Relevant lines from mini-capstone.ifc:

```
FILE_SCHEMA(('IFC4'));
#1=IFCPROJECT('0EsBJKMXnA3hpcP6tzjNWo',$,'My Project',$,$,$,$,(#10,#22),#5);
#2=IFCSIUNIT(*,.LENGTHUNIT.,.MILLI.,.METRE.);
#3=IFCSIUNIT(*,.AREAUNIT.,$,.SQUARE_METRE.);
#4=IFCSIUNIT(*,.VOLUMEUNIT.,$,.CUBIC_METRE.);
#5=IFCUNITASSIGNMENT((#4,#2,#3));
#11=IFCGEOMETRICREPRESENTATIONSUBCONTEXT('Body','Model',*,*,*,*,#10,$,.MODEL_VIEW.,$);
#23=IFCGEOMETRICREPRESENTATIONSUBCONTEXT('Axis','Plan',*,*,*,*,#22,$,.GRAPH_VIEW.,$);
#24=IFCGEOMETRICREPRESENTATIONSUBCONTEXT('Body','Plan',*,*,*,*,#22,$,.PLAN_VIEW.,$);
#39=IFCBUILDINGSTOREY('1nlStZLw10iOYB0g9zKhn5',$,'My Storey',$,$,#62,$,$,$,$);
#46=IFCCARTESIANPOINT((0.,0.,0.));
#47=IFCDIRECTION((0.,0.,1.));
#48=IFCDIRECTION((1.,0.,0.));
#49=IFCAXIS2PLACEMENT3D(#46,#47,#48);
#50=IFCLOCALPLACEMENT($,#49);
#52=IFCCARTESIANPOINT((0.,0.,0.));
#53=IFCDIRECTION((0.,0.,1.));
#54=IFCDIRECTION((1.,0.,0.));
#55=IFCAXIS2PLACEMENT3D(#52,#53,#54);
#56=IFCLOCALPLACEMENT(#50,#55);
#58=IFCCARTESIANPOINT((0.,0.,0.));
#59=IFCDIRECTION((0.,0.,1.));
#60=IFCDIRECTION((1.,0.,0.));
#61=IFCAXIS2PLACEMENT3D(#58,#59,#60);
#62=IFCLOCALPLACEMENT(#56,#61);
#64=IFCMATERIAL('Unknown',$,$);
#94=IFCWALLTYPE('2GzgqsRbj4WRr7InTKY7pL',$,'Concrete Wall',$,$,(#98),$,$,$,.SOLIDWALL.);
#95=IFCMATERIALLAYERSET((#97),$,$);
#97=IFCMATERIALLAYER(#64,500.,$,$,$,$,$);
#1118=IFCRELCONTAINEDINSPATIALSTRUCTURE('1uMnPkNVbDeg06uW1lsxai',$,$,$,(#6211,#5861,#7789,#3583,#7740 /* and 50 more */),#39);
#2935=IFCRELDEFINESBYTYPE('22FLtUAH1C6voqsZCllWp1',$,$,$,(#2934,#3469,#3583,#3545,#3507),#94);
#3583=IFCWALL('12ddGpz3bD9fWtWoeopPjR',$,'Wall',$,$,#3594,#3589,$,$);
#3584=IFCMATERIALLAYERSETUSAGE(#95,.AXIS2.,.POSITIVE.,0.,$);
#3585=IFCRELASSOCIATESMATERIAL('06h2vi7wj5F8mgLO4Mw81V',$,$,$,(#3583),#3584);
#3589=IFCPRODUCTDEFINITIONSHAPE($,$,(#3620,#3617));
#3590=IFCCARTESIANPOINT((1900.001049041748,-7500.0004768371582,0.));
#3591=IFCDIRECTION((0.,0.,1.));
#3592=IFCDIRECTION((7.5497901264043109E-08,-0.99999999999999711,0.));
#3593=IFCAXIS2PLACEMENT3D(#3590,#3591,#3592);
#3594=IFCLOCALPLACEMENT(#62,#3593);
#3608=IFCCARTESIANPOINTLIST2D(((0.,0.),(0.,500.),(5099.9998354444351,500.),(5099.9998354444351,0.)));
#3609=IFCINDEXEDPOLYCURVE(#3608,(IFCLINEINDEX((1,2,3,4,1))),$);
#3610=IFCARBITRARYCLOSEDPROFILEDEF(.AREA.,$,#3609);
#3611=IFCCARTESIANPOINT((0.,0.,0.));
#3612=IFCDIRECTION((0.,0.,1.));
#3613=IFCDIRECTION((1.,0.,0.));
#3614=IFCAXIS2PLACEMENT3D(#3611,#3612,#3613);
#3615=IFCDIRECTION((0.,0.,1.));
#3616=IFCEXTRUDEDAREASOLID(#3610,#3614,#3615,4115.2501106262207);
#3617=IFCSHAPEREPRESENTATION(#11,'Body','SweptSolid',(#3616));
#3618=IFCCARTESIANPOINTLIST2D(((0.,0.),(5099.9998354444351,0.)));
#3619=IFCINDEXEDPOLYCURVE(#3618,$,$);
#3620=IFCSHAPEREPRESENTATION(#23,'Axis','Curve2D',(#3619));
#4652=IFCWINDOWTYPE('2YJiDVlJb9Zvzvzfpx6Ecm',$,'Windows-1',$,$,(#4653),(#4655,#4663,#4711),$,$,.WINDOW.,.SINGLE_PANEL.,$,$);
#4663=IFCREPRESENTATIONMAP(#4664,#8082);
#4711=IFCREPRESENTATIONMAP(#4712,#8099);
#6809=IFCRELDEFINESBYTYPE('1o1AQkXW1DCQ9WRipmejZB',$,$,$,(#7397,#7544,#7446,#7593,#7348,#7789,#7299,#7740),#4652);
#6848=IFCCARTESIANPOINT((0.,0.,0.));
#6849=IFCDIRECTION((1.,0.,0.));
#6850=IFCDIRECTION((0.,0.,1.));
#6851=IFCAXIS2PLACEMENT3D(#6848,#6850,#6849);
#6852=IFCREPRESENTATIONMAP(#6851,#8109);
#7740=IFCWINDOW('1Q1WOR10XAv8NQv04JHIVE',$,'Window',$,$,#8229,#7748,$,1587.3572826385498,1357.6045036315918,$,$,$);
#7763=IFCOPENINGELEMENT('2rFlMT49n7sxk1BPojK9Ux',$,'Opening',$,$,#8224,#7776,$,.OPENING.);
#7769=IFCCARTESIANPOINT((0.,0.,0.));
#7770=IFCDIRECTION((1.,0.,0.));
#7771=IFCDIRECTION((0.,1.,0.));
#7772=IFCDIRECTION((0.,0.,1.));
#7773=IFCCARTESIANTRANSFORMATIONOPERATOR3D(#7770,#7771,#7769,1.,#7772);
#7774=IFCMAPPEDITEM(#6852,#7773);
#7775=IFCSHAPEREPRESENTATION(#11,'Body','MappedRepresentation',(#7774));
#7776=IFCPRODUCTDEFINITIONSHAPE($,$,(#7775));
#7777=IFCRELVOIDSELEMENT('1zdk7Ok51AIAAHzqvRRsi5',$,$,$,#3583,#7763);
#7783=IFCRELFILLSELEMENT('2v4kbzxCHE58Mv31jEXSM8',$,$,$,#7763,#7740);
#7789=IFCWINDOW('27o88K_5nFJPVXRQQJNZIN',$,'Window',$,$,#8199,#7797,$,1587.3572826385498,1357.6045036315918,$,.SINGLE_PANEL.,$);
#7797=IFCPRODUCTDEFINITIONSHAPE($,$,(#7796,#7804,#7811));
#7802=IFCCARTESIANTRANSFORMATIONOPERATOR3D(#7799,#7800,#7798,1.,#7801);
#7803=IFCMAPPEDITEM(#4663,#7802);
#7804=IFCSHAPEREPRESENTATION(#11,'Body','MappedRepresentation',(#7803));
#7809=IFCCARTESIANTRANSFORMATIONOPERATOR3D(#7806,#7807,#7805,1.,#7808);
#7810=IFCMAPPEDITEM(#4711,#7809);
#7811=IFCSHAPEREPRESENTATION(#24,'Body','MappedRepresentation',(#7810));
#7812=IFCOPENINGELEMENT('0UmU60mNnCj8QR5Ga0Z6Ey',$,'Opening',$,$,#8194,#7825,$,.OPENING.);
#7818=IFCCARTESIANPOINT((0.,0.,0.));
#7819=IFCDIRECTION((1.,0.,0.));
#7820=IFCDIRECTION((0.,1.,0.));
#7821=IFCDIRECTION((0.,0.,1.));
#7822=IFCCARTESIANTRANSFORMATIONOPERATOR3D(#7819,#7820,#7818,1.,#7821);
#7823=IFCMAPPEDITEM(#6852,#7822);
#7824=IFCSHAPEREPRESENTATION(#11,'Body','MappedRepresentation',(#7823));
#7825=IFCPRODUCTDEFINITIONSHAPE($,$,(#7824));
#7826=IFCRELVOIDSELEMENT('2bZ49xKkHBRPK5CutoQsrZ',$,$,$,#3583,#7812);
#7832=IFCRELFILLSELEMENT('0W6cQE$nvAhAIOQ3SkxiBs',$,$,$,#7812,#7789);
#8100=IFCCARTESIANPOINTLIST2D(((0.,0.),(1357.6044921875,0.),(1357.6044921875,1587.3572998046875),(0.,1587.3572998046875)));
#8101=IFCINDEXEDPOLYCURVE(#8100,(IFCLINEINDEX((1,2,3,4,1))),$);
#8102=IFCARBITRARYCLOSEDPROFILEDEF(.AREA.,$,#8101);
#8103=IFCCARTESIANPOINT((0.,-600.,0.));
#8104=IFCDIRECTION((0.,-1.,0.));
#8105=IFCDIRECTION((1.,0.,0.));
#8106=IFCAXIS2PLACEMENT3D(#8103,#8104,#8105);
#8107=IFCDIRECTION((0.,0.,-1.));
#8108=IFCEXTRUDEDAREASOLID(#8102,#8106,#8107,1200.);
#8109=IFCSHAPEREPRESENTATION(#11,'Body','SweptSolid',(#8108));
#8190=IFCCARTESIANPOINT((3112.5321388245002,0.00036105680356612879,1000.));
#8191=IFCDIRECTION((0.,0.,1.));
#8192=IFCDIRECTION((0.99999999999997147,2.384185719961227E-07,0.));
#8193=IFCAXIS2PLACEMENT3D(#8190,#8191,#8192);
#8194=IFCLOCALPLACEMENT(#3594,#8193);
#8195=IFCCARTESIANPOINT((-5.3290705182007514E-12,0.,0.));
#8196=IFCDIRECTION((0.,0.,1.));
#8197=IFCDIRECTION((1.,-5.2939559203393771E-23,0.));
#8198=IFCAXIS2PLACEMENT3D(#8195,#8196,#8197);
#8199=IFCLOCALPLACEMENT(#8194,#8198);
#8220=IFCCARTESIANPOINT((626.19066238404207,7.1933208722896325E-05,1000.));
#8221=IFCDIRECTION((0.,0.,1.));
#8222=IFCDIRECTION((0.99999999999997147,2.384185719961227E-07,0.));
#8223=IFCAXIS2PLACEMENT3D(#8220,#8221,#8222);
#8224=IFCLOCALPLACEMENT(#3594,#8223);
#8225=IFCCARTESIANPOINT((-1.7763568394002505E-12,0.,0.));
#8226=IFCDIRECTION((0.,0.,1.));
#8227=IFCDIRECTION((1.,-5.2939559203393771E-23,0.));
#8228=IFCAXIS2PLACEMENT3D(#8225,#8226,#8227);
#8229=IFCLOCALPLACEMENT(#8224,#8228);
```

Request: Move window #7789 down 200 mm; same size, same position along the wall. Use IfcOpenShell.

```python
import numpy as np
import ifcopenshell
import ifcopenshell.api.geometry
import ifcopenshell.util.placement
import ifcopenshell.util.unit

model = ifcopenshell.open("mini-capstone.ifc")
unit_scale = ifcopenshell.util.unit.calculate_unit_scale(model)

window = model.by_guid("27o88K_5nFJPVXRQQJNZIN")
opening = window.FillsVoids[0].RelatingOpeningElement
dz = -0.2 / unit_scale

shift = np.array([0.0, 0.0, dz])
# The window is placed relative to its opening, so it follows when the opening moves.
matrix = ifcopenshell.util.placement.get_local_placement(opening.ObjectPlacement)
matrix[:3, 3] += shift
ifcopenshell.api.geometry.edit_object_placement(
    model, product=opening, matrix=matrix, is_si=False, should_transform_children=True
)

print(f"moved by {dz * unit_scale:+.3f} m")

model.write("mini-capstone-out.ifc")
```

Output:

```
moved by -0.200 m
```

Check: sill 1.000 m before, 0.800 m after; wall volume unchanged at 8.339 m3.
